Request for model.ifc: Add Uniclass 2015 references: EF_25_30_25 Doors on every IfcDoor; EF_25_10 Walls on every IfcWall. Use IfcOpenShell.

First a look at what the model holds.

```python
import ifcopenshell

model = ifcopenshell.open("model.ifc")
print(model.schema)
print("classifications:", [c.Name for c in model.by_type("IfcClassification")])
for ifc_class in ("IfcDoor", "IfcRoof", "IfcStair", "IfcWall", "IfcWindow"):
    print(ifc_class, len(model.by_type(ifc_class)))
```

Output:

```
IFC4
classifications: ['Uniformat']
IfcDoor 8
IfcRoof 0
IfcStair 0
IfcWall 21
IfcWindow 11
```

```python
import ifcopenshell
import ifcopenshell.api.classification

model = ifcopenshell.open("model.ifc")

system = ifcopenshell.api.classification.add_classification(model, classification="Uniclass 2015")

codes = {
    "IfcDoor": ("EF_25_30_25", "Doors"),
    "IfcWall": ("EF_25_10", "Walls"),
}
for ifc_class, (code, name) in codes.items():
    products = model.by_type(ifc_class)
    ifcopenshell.api.classification.add_reference(
        model, products=products, classification=system, identification=code, name=name
    )
    print(code, len(products))

model.write("model_edited.ifc")
```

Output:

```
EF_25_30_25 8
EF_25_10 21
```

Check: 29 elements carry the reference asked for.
